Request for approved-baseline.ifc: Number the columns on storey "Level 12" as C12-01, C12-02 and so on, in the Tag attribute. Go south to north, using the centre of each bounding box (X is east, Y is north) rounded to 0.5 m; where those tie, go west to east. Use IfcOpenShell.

First a look at what the model holds.

```python
import ifcopenshell
import ifcopenshell.util.element
import ifcopenshell.util.placement

model = ifcopenshell.open("approved-baseline.ifc")
print(model.schema)
storey = next(s for s in model.by_type("IfcBuildingStorey") if s.Name == "Level 12")
columns = [e for e in ifcopenshell.util.element.get_decomposition(storey) if e.is_a("IfcColumn")]
for e in sorted(columns, key=lambda e: e.id()):
    origin = ifcopenshell.util.placement.get_local_placement(e.ObjectPlacement)[:3, 3]
    print(e.id(), e.Tag, e.Name, origin.round(2) + 0.0, sep=" | ")
```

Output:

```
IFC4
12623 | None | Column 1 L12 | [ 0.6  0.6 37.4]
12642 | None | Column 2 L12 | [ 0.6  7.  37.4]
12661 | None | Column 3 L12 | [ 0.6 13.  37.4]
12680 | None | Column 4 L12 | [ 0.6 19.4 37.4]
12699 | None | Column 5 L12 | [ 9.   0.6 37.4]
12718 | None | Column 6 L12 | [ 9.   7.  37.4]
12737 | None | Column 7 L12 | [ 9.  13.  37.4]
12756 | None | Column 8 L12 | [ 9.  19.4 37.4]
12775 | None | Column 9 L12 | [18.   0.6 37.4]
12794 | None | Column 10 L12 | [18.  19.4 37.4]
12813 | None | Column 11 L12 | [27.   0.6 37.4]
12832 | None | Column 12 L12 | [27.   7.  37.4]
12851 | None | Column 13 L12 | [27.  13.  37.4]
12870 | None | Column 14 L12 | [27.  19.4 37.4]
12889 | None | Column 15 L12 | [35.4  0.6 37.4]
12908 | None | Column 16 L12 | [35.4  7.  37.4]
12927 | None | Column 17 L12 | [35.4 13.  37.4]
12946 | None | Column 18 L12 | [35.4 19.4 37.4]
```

```python
import ifcopenshell
import ifcopenshell.geom
import ifcopenshell.util.element
import ifcopenshell.util.shape

model = ifcopenshell.open("approved-baseline.ifc")
settings = ifcopenshell.geom.settings()
settings.set("use-world-coords", True)


def centre(element):
    shape = ifcopenshell.geom.create_shape(settings, element)
    return ifcopenshell.util.shape.get_bbox_centroid(shape.geometry)


storey = next(s for s in model.by_type("IfcBuildingStorey") if s.Name == "Level 12")
columns = [e for e in ifcopenshell.util.element.get_decomposition(storey) if e.is_a("IfcColumn")]

# Insertion points can sit at a corner or the storey origin, so sort by the geometry (in metres).
centres = {e: centre(e) for e in columns}
columns.sort(key=lambda e: (round(centres[e][1] / 0.5), centres[e][0]))

for i, e in enumerate(columns, start=1):
    number = f"C12-{i:02d}"
    e.Tag = number
    print(e.id(), number)

model.write("approved-baseline-out.ifc")
```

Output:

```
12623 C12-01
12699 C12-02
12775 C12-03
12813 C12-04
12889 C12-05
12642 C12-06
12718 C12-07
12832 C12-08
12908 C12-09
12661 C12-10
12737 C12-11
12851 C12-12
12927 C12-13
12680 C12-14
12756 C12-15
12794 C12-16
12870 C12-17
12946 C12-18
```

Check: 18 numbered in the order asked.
